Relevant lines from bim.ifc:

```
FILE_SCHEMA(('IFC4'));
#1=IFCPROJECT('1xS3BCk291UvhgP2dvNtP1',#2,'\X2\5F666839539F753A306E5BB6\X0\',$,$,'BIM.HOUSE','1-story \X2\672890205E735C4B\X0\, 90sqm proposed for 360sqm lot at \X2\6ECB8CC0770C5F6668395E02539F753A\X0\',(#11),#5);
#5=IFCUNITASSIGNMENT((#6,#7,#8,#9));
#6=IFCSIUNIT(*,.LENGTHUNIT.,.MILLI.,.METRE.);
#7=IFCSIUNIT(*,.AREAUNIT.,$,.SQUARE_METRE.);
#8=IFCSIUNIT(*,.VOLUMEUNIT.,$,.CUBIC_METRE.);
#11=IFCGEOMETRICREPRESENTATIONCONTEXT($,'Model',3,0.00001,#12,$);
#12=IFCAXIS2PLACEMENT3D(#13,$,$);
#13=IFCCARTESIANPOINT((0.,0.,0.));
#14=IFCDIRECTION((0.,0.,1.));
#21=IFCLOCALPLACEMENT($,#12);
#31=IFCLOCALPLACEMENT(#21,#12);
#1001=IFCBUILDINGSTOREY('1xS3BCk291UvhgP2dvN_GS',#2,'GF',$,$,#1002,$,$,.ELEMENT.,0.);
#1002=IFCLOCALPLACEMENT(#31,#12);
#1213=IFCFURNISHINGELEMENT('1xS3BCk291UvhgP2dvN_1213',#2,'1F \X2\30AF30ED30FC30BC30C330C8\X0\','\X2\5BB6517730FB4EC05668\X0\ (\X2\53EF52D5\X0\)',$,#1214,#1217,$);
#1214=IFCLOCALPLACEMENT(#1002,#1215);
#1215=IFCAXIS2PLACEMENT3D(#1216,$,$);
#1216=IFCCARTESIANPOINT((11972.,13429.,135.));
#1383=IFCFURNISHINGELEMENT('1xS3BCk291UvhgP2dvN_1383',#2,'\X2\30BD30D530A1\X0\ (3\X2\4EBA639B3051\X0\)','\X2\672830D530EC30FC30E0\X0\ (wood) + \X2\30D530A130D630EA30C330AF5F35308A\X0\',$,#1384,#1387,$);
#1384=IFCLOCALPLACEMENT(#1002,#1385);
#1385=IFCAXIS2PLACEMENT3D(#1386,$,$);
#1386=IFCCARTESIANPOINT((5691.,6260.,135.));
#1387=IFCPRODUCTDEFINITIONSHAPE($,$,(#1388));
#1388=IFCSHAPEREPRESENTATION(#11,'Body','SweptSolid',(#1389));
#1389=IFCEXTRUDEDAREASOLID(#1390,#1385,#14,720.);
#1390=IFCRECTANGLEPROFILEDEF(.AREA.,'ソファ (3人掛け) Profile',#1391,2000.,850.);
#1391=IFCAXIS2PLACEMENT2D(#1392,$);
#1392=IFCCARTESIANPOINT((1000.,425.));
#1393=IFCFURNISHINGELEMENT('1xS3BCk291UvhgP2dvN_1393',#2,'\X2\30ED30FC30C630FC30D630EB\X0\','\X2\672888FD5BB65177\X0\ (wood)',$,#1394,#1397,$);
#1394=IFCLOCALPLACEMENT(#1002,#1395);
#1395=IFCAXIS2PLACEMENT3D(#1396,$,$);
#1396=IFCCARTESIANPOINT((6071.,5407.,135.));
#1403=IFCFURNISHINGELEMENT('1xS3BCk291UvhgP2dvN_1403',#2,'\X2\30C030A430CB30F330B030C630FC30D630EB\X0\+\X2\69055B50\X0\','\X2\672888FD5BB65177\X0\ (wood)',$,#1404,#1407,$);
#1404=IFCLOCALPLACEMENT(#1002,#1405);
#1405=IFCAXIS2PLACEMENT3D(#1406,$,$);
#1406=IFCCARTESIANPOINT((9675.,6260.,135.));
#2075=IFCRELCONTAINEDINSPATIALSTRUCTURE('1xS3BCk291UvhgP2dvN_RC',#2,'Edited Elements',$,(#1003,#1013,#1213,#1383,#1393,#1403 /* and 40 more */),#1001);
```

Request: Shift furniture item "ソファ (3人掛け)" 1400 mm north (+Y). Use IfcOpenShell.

```python
import ifcopenshell
import ifcopenshell.api.geometry
import ifcopenshell.util.placement
import ifcopenshell.util.unit

model = ifcopenshell.open("bim.ifc")
unit_scale = ifcopenshell.util.unit.calculate_unit_scale(model)

item = model.by_id(1383)
matrix = ifcopenshell.util.placement.get_local_placement(item.ObjectPlacement)
matrix[1, 3] += 1.4 / unit_scale
ifcopenshell.api.geometry.edit_object_placement(model, product=item, matrix=matrix, is_si=False)

print(ifcopenshell.util.placement.get_local_placement(item.ObjectPlacement).round(3) + 0.0)

model.write("bim_v2.ifc")
```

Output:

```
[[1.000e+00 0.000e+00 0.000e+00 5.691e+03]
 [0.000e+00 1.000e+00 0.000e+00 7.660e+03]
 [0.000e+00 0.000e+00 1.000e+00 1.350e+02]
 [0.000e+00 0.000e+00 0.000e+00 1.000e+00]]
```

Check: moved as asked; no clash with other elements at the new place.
